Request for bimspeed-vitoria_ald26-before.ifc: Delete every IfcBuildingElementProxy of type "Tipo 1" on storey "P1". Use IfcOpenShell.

First a look at what the model holds.

```python
import ifcopenshell
import ifcopenshell.util.element

model = ifcopenshell.open("bimspeed-vitoria_ald26-before.ifc")
print(model.schema)
storey = next(s for s in model.by_type("IfcBuildingStorey") if s.Name == "P1")
proxies = [e for e in ifcopenshell.util.element.get_decomposition(storey) if e.is_a("IfcBuildingElementProxy")]
seen = {}
for e in proxies:
    element_type = ifcopenshell.util.element.get_type(e)
    name = element_type.Name if element_type not in (None, e) else None
    seen[name] = seen.get(name, 0) + 1
for name, count in sorted(seen.items(), key=str):
    print(count, "x", name)
```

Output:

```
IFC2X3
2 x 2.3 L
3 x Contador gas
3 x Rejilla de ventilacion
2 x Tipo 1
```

```python
import ifcopenshell
import ifcopenshell.api.root
import ifcopenshell.util.element

model = ifcopenshell.open("bimspeed-vitoria_ald26-before.ifc")

storey = next(s for s in model.by_type("IfcBuildingStorey") if s.Name == "P1")
proxies = [e for e in ifcopenshell.util.element.get_decomposition(storey) if e.is_a("IfcBuildingElementProxy")]
targets = [e for e in proxies if (t := ifcopenshell.util.element.get_type(e)) not in (None, e) and t.Name == "Tipo 1"]

for e in targets:
    ifcopenshell.api.root.remove_product(model, product=e)
print(len(targets), "removed")

model.write("bimspeed-vitoria_ald26-before_edited.ifc")
```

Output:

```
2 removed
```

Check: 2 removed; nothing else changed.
